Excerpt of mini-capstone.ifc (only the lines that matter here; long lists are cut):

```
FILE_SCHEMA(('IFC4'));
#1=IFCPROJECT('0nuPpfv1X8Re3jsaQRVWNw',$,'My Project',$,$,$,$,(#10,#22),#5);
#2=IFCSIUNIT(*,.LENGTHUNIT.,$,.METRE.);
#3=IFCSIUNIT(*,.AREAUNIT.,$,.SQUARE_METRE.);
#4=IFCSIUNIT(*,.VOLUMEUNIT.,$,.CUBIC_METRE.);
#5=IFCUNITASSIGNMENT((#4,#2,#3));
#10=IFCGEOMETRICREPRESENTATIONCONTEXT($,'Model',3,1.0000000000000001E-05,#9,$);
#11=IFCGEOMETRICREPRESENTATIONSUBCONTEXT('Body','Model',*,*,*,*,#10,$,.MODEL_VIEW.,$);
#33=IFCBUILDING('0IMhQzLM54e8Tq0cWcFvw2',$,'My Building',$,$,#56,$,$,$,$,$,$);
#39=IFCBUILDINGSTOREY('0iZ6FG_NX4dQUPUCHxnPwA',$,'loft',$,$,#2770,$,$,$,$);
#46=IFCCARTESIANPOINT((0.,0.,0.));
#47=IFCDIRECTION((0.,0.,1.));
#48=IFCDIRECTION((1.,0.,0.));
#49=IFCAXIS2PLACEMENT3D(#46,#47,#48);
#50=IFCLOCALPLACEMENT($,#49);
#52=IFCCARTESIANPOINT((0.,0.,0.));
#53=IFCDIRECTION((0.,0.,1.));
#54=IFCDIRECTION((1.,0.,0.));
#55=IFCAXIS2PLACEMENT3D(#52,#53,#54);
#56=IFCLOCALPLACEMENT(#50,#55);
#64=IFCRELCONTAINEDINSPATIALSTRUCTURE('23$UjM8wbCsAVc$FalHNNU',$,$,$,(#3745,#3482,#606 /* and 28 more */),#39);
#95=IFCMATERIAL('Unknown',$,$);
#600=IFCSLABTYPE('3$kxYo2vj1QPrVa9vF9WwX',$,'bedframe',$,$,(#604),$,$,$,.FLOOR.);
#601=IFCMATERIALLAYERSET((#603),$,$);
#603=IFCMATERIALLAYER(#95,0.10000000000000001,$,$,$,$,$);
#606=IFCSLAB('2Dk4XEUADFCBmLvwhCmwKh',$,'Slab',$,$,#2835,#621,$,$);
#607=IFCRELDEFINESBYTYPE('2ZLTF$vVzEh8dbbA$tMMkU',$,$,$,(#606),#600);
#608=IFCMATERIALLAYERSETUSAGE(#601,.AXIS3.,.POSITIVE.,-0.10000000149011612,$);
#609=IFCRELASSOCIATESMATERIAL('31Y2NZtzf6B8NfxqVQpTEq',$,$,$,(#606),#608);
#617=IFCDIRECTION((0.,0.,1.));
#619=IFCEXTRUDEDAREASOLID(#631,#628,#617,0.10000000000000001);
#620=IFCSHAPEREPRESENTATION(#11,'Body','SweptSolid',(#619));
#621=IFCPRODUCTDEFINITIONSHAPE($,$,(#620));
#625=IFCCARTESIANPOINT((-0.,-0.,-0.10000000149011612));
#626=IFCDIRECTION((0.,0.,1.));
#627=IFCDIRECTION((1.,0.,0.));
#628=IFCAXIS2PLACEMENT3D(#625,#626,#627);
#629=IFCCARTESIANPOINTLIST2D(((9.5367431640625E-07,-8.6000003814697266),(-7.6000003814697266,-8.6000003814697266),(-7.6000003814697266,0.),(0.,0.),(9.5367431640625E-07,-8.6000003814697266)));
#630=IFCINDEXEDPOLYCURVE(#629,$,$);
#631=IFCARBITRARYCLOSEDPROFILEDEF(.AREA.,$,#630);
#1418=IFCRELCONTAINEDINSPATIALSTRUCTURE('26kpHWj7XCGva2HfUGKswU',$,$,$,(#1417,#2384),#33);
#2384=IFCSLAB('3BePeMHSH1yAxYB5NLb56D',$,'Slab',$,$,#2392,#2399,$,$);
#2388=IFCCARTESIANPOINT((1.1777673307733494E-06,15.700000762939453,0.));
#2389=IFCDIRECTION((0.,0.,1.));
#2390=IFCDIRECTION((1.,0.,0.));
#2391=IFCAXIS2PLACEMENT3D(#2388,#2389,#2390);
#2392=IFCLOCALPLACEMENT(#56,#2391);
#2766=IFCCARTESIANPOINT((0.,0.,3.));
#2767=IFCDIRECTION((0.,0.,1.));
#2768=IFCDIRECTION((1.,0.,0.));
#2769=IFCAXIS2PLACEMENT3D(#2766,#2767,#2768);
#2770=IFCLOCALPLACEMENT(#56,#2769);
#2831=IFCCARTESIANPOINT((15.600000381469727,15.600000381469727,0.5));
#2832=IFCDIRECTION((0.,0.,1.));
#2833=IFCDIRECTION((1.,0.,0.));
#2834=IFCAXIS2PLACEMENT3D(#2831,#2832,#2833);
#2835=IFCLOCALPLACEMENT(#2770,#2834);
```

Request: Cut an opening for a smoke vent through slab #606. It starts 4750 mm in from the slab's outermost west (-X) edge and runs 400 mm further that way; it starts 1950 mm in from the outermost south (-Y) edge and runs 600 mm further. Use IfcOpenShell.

```python
import numpy as np
import ifcopenshell
import ifcopenshell.api.feature
import ifcopenshell.api.geometry
import ifcopenshell.api.root
import ifcopenshell.geom
import ifcopenshell.util.placement
import ifcopenshell.util.representation
import ifcopenshell.util.shape
import ifcopenshell.util.unit

model = ifcopenshell.open("mini-capstone.ifc")
unit_scale = ifcopenshell.util.unit.calculate_unit_scale(model)
settings = ifcopenshell.geom.settings()


def volume(element):
    """Net volume in cubic metres, openings subtracted."""
    shape = ifcopenshell.geom.create_shape(settings, element)
    return ifcopenshell.util.shape.get_volume(shape.geometry)


slab = model.by_guid("2Dk4XEUADFCBmLvwhCmwKh")
before = volume(slab)

# Extent in the slab's own axes, in metres. The edges named are its -X and -Y sides.
slab_shape = ifcopenshell.geom.create_shape(settings, slab)
vertices = ifcopenshell.util.shape.get_vertices(slab_shape.geometry)
x_min, y_min, bottom = vertices.min(axis=0)
top = vertices[:, 2].max()

opening = ifcopenshell.api.root.create_entity(model, ifc_class="IfcOpeningElement", name="Smoke vent opening", predefined_type="OPENING")
context = ifcopenshell.util.representation.get_context(model, "Model", "Body", "MODEL_VIEW")
width, depth = 0.4, 0.6
outline = [(0.0, 0.0), (width, 0.0), (width, depth), (0.0, depth), (0.0, 0.0)]
# Overshoot both faces by 50 mm so the cut is clean.
shape = ifcopenshell.api.geometry.add_slab_representation(
    model, context=context, depth=top - bottom + 0.1, polyline=outline
)
ifcopenshell.api.geometry.assign_representation(model, product=opening, representation=shape)

matrix = ifcopenshell.util.placement.get_local_placement(slab.ObjectPlacement)
matrix[:, 3] = matrix @ np.append(np.array([x_min + 4.75, y_min + 1.95, bottom - 0.05]) / unit_scale, 1.0)
ifcopenshell.api.geometry.edit_object_placement(model, product=opening, matrix=matrix, is_si=False)
ifcopenshell.api.feature.add_feature(model, feature=opening, element=slab)

after = volume(slab)

print(f"slab volume {before:.3f} -> {after:.3f} m3")

model.write("mini-capstone-out.ifc")
```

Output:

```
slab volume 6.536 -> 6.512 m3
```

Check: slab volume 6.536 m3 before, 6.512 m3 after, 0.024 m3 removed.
